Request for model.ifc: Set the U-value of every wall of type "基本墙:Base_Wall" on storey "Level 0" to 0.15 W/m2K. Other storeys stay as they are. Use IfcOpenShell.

First a look at what the model holds.

```python
import ifcopenshell
import ifcopenshell.util.element

model = ifcopenshell.open("model.ifc")
print(model.schema)
storey = next(s for s in model.by_type("IfcBuildingStorey") if s.Name == "Level 0")
walls = [e for e in ifcopenshell.util.element.get_decomposition(storey) if e.is_a("IfcWall")]
seen = {}
for e in walls:
    element_type = ifcopenshell.util.element.get_type(e)
    key = (element_type.Name if element_type != e and element_type else None, ifcopenshell.util.element.get_pset(e, "Pset_WallCommon", "ThermalTransmittance"))
    seen[key] = seen.get(key, 0) + 1
for (name, value), count in sorted(seen.items(), key=str):
    print(count, "x", name, "|", value)
```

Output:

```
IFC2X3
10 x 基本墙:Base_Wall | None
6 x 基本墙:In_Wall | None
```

```python
import ifcopenshell
import ifcopenshell.api.pset
import ifcopenshell.util.element

model = ifcopenshell.open("model.ifc")

storey = next(s for s in model.by_type("IfcBuildingStorey") if s.Name == "Level 0")
walls = [e for e in ifcopenshell.util.element.get_decomposition(storey) if e.is_a("IfcWall")]

count = 0
for e in walls:
    element_type = ifcopenshell.util.element.get_type(e)
    if element_type in (None, e) or element_type.Name != "基本墙:Base_Wall":
        continue
    # add_pset returns the element's existing set when there is one.
    pset = ifcopenshell.api.pset.add_pset(model, product=e, name="Pset_WallCommon")
    ifcopenshell.api.pset.edit_pset(model, pset=pset, properties={"ThermalTransmittance": 0.15})
    count += 1

print(count, "walls updated")

model.write("model_rev.ifc")
```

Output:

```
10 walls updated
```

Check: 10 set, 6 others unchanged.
